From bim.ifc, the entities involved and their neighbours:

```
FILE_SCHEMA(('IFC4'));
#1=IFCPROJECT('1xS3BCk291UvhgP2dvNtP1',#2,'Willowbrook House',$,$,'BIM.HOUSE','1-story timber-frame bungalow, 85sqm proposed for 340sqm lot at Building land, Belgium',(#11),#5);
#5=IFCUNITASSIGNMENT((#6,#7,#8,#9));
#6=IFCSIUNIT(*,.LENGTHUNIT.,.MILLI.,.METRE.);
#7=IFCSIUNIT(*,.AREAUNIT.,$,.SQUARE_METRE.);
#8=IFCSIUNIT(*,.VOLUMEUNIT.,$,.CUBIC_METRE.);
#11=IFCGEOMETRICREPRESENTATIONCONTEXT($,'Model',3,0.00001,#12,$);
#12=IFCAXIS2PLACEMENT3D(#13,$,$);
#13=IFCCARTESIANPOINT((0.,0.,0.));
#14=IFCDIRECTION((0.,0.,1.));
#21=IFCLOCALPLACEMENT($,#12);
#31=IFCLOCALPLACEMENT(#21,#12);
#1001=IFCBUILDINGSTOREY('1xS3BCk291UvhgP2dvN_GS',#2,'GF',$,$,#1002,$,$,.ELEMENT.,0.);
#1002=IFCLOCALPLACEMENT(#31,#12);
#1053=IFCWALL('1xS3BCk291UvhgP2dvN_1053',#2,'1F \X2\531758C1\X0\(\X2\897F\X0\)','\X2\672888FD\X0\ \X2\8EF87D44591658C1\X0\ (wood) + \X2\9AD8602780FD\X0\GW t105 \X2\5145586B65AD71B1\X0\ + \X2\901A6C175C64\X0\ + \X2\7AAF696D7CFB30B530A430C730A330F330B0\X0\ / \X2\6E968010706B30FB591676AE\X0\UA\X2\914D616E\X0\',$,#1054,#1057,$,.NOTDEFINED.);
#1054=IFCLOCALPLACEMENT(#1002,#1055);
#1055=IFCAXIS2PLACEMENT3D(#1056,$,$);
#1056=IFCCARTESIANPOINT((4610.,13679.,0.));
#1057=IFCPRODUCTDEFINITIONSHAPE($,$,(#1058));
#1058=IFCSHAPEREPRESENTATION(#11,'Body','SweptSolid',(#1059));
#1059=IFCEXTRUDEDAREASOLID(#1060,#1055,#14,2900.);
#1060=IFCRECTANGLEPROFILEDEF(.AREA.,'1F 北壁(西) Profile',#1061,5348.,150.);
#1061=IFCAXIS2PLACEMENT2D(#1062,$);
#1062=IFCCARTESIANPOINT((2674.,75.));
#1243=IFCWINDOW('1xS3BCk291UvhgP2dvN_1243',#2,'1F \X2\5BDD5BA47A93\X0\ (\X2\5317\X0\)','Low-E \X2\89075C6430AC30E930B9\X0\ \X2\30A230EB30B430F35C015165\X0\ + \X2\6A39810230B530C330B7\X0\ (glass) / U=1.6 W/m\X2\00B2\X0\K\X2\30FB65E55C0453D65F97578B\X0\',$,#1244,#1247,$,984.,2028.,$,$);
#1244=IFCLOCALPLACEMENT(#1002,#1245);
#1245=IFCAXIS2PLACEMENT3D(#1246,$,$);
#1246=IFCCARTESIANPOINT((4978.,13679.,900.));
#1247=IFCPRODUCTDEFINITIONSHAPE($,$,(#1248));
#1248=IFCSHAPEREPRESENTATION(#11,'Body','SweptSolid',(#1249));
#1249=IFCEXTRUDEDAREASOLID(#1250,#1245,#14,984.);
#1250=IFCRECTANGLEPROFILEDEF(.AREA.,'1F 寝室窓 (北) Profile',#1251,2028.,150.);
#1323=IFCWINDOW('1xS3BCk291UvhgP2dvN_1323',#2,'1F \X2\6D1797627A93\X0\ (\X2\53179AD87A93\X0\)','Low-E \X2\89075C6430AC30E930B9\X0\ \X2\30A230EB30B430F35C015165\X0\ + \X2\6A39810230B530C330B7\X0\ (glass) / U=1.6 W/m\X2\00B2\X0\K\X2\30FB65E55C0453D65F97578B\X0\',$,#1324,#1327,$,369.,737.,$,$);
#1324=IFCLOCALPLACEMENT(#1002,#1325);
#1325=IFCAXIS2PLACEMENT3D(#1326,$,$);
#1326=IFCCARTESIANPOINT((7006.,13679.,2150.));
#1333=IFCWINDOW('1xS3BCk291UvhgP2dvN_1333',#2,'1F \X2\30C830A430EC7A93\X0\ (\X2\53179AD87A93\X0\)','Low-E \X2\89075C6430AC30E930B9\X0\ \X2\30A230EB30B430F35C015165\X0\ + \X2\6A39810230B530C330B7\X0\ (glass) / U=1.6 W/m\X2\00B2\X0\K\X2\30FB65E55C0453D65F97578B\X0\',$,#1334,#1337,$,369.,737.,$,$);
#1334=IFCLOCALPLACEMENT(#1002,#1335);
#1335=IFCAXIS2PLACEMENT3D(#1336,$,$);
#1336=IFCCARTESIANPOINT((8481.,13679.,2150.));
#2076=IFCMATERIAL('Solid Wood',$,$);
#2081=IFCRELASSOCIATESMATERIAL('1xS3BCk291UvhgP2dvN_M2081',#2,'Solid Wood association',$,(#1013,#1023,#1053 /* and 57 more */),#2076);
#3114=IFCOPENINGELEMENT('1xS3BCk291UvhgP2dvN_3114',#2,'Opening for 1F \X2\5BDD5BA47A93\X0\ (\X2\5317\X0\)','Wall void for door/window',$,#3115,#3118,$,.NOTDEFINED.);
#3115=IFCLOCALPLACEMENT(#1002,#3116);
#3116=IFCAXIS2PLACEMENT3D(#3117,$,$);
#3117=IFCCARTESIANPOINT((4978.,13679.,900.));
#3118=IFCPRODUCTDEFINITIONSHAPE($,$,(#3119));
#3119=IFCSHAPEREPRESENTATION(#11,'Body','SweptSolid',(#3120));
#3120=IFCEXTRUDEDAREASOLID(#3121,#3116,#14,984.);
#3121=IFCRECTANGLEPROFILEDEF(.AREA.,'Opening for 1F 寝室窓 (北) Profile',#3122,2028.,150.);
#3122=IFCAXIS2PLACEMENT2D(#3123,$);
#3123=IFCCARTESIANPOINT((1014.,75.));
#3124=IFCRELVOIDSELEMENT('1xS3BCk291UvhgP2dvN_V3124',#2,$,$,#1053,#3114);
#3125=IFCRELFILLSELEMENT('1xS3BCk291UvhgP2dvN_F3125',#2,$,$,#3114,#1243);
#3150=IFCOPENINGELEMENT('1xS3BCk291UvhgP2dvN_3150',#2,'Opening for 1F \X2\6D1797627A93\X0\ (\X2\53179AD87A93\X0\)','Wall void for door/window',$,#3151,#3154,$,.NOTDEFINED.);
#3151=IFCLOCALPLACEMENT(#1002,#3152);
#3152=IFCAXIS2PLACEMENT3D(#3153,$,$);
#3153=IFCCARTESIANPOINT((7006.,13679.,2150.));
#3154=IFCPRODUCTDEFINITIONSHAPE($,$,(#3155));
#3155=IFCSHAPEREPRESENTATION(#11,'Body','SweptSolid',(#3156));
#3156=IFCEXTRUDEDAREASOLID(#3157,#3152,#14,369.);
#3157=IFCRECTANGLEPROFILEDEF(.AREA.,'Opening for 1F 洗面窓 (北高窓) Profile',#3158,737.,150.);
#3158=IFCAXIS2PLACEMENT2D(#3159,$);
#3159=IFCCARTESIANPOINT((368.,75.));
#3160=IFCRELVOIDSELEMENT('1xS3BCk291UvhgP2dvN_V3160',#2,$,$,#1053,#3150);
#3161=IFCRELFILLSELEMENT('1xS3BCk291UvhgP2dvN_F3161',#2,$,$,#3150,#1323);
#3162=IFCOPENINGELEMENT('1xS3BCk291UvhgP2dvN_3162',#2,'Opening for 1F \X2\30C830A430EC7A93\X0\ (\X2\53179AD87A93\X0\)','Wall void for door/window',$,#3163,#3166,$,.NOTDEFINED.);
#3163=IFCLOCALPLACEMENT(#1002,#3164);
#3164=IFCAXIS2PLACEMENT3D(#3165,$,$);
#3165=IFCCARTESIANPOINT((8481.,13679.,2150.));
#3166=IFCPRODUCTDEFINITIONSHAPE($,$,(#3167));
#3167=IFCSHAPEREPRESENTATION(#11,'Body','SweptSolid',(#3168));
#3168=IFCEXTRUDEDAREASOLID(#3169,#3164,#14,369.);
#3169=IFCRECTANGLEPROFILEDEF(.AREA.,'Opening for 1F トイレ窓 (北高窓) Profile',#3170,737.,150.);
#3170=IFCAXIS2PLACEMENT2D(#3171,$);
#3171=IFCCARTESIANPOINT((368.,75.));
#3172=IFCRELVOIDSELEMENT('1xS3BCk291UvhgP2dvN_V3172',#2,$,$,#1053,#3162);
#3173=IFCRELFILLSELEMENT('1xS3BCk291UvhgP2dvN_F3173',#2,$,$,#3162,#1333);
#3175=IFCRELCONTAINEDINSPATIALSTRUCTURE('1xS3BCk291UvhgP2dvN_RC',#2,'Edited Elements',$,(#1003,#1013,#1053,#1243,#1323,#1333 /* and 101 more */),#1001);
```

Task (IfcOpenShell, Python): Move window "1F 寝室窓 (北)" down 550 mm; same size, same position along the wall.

```python
import numpy as np
import ifcopenshell
import ifcopenshell.api.geometry
import ifcopenshell.util.placement
import ifcopenshell.util.unit

model = ifcopenshell.open("bim.ifc")
unit_scale = ifcopenshell.util.unit.calculate_unit_scale(model)

window = model.by_id(1243)
opening = window.FillsVoids[0].RelatingOpeningElement
dz = -550.0

shift = np.array([0.0, 0.0, dz])
# The window is not placed relative to its opening, so move both.
for product in (opening, window):
    matrix = ifcopenshell.util.placement.get_local_placement(product.ObjectPlacement)
    matrix[:3, 3] += shift
    ifcopenshell.api.geometry.edit_object_placement(model, product=product, matrix=matrix, is_si=False)

print(f"moved by {dz * unit_scale:+.3f} m")

model.write("bim_rev.ifc")
```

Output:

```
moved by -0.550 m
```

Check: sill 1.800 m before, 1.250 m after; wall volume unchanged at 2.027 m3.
